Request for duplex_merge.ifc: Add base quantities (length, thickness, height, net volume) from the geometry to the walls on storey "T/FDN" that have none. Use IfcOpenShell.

First a look at what the model holds.

```python
import ifcopenshell
import ifcopenshell.util.element
import ifcopenshell.util.unit

model = ifcopenshell.open("duplex_merge.ifc")
print(model.schema)
for unit_type in ("LENGTHUNIT", "AREAUNIT", "VOLUMEUNIT"):
    print(unit_type, ifcopenshell.util.unit.calculate_unit_scale(model, unit_type))
storey = next(s for s in model.by_type("IfcBuildingStorey") if s.Name == "T/FDN")
walls = [e for e in ifcopenshell.util.element.get_decomposition(storey) if e.is_a("IfcWall")]
for e in sorted(walls, key=lambda e: e.id()):
    print(e.id(), e.is_a(), e.Name, list(ifcopenshell.util.element.get_psets(e, qtos_only=True)), sep=" | ")
```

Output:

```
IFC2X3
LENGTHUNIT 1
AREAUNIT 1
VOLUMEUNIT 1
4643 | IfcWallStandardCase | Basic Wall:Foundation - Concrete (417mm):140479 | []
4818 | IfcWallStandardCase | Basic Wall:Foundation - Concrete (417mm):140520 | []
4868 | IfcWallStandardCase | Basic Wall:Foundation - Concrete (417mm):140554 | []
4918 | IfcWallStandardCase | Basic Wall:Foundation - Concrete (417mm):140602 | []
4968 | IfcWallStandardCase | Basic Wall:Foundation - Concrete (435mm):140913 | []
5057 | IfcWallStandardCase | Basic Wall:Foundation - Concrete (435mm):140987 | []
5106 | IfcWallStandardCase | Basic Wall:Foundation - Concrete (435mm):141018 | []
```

```python
import ifcopenshell
import ifcopenshell.api.pset
import ifcopenshell.geom
import ifcopenshell.util.element
import ifcopenshell.util.shape
import ifcopenshell.util.unit

model = ifcopenshell.open("duplex_merge.ifc")
unit_scale = ifcopenshell.util.unit.calculate_unit_scale(model)
volume_scale = ifcopenshell.util.unit.calculate_unit_scale(model, "VOLUMEUNIT")
settings = ifcopenshell.geom.settings()

storey = next(s for s in model.by_type("IfcBuildingStorey") if s.Name == "T/FDN")
walls = [e for e in ifcopenshell.util.element.get_decomposition(storey) if e.is_a("IfcWall")]

for e in sorted(walls, key=lambda e: e.id()):
    if ifcopenshell.util.element.get_psets(e, qtos_only=True, should_inherit=False):
        continue
    # Geometry comes back in metres, in the element's own axes.
    shape = ifcopenshell.geom.create_shape(settings, e)
    values = {
        "Length": ifcopenshell.util.shape.get_x(shape.geometry) / unit_scale,
        "Width": ifcopenshell.util.shape.get_y(shape.geometry) / unit_scale,
        "Height": ifcopenshell.util.shape.get_z(shape.geometry) / unit_scale,
        "NetVolume": ifcopenshell.util.shape.get_volume(shape.geometry) / volume_scale,
    }
    qto = ifcopenshell.api.pset.add_qto(model, product=e, name="BaseQuantities")
    ifcopenshell.api.pset.edit_qto(model, qto=qto, properties=values)
    print(e.id(), {k: round(v, 3) for k, v in values.items()})

model.write("duplex_merge_rev.ifc")
```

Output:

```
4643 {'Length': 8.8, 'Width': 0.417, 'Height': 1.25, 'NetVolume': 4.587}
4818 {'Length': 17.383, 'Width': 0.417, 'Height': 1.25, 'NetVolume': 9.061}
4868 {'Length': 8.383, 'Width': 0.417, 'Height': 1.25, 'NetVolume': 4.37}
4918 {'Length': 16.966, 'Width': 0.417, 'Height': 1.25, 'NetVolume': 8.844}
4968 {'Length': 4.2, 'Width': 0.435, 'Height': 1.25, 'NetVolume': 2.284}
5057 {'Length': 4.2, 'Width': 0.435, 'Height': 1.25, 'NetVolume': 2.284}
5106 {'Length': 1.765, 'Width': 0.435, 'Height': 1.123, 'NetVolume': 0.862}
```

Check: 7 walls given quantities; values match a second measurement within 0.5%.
